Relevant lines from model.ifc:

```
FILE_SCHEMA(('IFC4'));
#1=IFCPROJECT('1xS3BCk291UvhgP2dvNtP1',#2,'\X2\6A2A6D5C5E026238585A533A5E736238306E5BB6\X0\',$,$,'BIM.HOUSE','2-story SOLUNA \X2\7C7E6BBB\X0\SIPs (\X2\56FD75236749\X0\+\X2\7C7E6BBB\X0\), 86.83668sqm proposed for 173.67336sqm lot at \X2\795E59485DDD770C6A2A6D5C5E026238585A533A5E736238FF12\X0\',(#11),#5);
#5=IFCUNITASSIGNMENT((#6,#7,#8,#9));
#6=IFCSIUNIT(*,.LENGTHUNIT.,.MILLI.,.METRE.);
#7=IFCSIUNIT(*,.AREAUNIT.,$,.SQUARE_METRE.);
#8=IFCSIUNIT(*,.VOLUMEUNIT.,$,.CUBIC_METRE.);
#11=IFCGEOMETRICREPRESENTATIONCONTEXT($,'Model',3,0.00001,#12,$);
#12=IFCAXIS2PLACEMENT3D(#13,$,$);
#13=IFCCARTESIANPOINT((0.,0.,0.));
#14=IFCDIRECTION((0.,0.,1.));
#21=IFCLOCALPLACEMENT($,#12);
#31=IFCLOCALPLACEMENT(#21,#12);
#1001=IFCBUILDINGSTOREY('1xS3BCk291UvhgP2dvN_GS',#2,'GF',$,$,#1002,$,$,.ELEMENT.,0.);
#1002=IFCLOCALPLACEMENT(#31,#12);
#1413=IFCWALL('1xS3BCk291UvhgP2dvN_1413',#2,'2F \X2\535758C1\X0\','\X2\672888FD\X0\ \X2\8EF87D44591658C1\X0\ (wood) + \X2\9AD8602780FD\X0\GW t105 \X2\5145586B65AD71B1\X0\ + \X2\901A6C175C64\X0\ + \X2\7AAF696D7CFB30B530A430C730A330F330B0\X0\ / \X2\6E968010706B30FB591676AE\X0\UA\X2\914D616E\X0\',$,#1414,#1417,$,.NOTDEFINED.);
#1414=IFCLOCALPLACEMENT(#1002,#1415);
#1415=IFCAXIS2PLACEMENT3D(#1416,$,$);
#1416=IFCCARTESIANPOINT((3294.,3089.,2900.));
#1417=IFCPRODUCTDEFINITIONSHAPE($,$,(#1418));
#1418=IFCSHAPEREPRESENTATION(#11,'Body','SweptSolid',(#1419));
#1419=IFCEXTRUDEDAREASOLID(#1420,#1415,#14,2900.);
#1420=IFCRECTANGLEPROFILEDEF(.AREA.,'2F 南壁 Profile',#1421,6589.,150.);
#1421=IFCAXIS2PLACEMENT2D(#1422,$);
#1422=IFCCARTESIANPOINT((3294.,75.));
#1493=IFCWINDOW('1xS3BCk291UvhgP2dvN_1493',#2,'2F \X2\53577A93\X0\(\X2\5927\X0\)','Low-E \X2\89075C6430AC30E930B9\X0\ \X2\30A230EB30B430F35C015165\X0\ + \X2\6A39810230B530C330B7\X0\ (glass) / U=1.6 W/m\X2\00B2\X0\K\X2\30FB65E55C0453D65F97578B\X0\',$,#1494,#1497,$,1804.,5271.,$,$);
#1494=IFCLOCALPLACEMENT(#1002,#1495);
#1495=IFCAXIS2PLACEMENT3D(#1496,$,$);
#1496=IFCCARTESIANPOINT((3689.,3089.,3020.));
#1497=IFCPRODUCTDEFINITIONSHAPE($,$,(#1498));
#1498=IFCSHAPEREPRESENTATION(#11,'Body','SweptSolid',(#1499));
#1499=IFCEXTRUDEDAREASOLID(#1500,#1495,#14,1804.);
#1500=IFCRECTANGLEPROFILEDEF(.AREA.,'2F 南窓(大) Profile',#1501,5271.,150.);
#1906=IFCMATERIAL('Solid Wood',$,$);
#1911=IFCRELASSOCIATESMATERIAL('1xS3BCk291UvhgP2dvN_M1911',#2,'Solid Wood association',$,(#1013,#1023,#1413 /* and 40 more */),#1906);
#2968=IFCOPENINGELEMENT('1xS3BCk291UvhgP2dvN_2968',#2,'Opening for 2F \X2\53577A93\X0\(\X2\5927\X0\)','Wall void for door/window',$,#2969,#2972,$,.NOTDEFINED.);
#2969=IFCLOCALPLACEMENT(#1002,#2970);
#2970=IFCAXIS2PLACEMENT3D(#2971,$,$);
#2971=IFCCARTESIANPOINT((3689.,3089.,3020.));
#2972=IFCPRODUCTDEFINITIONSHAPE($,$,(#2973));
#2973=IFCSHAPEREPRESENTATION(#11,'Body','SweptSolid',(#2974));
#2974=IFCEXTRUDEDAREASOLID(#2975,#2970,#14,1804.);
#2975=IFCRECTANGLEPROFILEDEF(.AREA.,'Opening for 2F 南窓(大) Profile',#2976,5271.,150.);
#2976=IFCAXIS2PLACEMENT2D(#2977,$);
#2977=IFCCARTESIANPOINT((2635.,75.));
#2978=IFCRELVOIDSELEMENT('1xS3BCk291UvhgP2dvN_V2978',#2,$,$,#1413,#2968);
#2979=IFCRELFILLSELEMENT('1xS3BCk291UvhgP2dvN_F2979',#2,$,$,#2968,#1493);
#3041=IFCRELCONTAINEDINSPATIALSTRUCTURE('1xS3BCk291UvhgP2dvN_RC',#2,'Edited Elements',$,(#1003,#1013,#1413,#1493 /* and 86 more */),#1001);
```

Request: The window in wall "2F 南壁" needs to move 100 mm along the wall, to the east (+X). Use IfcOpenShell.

```python
import ifcopenshell
import ifcopenshell.api.geometry
import ifcopenshell.util.placement

model = ifcopenshell.open("model.ifc")

window = model.by_guid("1xS3BCk291UvhgP2dvN_1493")
opening = window.FillsVoids[0].RelatingOpeningElement
wall = opening.VoidsElements[0].RelatingBuildingElement

wall_matrix = ifcopenshell.util.placement.get_local_placement(wall.ObjectPlacement)
shift = wall_matrix[:3, 0] * 100.0
before = ifcopenshell.util.placement.get_local_placement(window.ObjectPlacement)[:3, 3].copy()

# The window is not placed relative to its opening, so move both.
for product in (opening, window):
    matrix = ifcopenshell.util.placement.get_local_placement(product.ObjectPlacement)
    matrix[:3, 3] += shift
    ifcopenshell.api.geometry.edit_object_placement(model, product=product, matrix=matrix, is_si=False)

after = ifcopenshell.util.placement.get_local_placement(window.ObjectPlacement)[:3, 3]
print("window moved by", (after - before).round(3) + 0.0)

model.write("model_updated.ifc")
```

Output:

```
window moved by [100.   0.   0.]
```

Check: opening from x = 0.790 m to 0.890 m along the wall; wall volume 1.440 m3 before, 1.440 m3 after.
